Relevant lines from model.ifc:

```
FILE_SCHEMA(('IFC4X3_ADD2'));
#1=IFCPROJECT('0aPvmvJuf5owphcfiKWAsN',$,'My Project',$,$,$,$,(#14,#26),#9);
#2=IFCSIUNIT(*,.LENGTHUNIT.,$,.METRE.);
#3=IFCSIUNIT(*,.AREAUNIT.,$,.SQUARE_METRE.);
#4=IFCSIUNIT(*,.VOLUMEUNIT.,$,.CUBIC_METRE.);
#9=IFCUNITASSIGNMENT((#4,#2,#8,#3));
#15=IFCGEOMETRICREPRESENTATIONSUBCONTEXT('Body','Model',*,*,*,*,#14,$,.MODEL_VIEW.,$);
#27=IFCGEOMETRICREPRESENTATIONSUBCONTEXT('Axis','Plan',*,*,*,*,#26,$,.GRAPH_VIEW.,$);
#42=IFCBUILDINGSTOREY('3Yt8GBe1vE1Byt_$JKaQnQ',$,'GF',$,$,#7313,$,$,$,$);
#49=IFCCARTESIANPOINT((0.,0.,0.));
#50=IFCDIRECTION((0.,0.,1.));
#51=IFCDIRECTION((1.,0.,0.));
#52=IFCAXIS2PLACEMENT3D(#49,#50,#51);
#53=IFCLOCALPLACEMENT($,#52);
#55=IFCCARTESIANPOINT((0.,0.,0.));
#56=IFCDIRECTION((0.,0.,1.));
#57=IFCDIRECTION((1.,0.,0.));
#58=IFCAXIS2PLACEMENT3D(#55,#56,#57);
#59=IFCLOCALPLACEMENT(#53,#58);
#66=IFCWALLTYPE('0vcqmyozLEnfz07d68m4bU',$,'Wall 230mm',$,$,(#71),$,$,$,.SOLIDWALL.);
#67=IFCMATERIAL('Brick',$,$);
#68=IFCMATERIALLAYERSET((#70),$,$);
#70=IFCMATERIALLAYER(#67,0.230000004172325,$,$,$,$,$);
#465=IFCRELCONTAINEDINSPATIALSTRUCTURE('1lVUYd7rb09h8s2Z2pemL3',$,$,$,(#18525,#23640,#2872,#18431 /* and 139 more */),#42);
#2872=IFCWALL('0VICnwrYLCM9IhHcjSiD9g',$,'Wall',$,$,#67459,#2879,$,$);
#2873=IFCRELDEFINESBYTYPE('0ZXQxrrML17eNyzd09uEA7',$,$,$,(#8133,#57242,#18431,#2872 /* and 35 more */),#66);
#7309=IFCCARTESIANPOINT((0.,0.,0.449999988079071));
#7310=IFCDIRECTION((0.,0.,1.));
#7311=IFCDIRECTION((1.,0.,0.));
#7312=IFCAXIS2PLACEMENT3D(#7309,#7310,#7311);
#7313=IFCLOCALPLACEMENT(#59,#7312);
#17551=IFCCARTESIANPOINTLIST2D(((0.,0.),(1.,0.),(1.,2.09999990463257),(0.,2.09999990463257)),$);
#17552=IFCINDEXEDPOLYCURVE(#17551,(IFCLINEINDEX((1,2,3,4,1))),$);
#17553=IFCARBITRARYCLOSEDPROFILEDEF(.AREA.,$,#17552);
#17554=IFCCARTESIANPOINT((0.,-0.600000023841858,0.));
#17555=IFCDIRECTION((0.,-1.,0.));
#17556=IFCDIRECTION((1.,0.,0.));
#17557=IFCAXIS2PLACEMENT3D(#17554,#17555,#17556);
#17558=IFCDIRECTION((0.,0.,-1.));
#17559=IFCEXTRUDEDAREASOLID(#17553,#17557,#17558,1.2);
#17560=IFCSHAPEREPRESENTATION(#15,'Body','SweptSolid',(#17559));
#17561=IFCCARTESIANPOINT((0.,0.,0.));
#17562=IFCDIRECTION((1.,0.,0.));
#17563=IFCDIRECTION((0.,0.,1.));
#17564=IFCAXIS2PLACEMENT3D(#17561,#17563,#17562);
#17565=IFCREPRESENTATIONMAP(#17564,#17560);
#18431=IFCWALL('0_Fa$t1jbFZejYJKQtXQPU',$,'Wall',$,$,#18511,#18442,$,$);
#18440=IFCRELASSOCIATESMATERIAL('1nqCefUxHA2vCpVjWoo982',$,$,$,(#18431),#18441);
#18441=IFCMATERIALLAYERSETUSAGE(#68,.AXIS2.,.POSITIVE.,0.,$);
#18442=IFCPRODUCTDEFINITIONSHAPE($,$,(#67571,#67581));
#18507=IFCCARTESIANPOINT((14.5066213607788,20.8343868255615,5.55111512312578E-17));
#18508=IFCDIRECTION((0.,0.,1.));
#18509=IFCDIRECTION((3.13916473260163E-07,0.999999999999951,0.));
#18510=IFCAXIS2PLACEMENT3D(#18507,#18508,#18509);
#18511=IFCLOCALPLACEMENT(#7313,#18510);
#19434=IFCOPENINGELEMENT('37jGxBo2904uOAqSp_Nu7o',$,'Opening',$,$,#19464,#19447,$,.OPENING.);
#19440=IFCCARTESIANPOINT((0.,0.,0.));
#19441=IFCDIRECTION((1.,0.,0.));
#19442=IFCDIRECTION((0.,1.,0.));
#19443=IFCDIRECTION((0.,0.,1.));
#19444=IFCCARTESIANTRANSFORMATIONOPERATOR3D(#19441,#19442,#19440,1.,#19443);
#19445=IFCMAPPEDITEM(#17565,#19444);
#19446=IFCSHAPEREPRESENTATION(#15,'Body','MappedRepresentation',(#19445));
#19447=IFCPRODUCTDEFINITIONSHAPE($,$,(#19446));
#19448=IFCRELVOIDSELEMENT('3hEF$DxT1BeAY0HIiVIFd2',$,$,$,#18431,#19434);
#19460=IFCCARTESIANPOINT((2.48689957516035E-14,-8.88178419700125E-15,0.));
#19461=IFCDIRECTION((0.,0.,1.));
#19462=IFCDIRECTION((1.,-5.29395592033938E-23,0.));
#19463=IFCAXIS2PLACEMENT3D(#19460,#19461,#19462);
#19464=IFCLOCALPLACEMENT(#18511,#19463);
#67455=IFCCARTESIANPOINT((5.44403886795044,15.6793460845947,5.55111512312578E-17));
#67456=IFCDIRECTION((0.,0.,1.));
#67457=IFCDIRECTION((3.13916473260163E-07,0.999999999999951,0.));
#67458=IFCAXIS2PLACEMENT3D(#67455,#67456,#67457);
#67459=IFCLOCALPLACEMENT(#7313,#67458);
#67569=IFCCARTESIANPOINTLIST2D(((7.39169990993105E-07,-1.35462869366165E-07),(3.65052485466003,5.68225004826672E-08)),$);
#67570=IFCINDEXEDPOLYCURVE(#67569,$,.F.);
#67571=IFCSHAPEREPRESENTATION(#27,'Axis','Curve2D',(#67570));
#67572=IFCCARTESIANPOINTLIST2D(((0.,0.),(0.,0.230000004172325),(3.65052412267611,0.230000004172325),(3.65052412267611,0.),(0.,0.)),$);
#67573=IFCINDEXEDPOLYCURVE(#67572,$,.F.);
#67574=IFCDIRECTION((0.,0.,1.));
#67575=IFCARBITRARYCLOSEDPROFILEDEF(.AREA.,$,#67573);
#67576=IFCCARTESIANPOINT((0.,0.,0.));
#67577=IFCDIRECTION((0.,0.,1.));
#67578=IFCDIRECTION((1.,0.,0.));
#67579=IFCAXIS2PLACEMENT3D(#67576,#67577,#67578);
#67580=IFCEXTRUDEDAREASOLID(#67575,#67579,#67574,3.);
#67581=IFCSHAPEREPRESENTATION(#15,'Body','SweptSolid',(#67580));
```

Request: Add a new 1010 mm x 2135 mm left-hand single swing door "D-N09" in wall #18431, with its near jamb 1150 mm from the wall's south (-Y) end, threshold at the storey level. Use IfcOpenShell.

```python
import numpy as np
import ifcopenshell
import ifcopenshell.api.feature
import ifcopenshell.api.geometry
import ifcopenshell.api.root
import ifcopenshell.api.spatial
import ifcopenshell.geom
import ifcopenshell.util.element
import ifcopenshell.util.placement
import ifcopenshell.util.representation
import ifcopenshell.util.shape
import ifcopenshell.util.unit

model = ifcopenshell.open("model.ifc")
unit_scale = ifcopenshell.util.unit.calculate_unit_scale(model)
settings = ifcopenshell.geom.settings()


def volume(element):
    """Net volume in cubic metres, openings subtracted."""
    shape = ifcopenshell.geom.create_shape(settings, element)
    return ifcopenshell.util.shape.get_volume(shape.geometry)


wall = model.by_guid("0_Fa$t1jbFZejYJKQtXQPU")
storey = ifcopenshell.util.element.get_container(wall, ifc_class="IfcBuildingStorey")
context = ifcopenshell.util.representation.get_context(model, "Model", "Body", "MODEL_VIEW")
before = volume(wall)

width, height, from_end, sill = 1.01, 2.135, 1.15, 0.0  # metres

# The wall runs along its own X axis, and the end named is its -X end.
wall_shape = ifcopenshell.geom.create_shape(settings, wall)
x, y, z = ifcopenshell.util.shape.get_vertices(wall_shape.geometry).T
start = x.min() + from_end
face, thickness = float(y.min()), float(y.max() - y.min())
wall_matrix = ifcopenshell.util.placement.get_local_placement(wall.ObjectPlacement)
level = ifcopenshell.util.placement.get_local_placement(storey.ObjectPlacement)[2, 3]


def in_wall(x, y):
    """Placement at x, y metres in the wall's axes, at sill height."""
    matrix = wall_matrix.copy()
    matrix[:, 3] = wall_matrix @ np.array([x / unit_scale, y / unit_scale, 0.0, 1.0])
    matrix[2, 3] = level + sill / unit_scale
    return matrix


# Opening: a box that overshoots both wall faces by 50 mm.
opening = ifcopenshell.api.root.create_entity(model, ifc_class="IfcOpeningElement", predefined_type="OPENING")
box = ifcopenshell.api.geometry.add_wall_representation(
    model, context=context, length=width, height=height, thickness=thickness + 0.1
)
ifcopenshell.api.geometry.assign_representation(model, product=opening, representation=box)
ifcopenshell.api.geometry.edit_object_placement(model, product=opening, matrix=in_wall(start, face - 0.05), is_si=False)
ifcopenshell.api.feature.add_feature(model, feature=opening, element=wall)

door = ifcopenshell.api.root.create_entity(model, ifc_class="IfcDoor", name="D-N09", predefined_type="DOOR")
door.OverallWidth, door.OverallHeight = width / unit_scale, height / unit_scale
door.OperationType = "SINGLE_SWING_LEFT"
body = ifcopenshell.api.geometry.add_door_representation(
    model,
    context=context,
    overall_width=door.OverallWidth,
    overall_height=door.OverallHeight,
    operation_type="SINGLE_SWING_LEFT",
    lining_properties={"LiningDepth": thickness / unit_scale, "ThresholdDepth": thickness / unit_scale},
)
ifcopenshell.api.geometry.assign_representation(model, product=door, representation=body)
ifcopenshell.api.spatial.assign_container(model, products=[door], relating_structure=storey)
ifcopenshell.api.feature.add_filling(model, opening=opening, element=door)

# The lining spans the wall, so the door starts at the wall face.
ifcopenshell.api.geometry.edit_object_placement(model, product=door, matrix=in_wall(start, face), is_si=False)

after = volume(wall)

print(f"wall volume {before:.3f} -> {after:.3f} m3")

model.write("model_edited.ifc")
```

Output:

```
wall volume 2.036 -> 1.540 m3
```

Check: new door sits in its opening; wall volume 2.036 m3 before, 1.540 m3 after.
